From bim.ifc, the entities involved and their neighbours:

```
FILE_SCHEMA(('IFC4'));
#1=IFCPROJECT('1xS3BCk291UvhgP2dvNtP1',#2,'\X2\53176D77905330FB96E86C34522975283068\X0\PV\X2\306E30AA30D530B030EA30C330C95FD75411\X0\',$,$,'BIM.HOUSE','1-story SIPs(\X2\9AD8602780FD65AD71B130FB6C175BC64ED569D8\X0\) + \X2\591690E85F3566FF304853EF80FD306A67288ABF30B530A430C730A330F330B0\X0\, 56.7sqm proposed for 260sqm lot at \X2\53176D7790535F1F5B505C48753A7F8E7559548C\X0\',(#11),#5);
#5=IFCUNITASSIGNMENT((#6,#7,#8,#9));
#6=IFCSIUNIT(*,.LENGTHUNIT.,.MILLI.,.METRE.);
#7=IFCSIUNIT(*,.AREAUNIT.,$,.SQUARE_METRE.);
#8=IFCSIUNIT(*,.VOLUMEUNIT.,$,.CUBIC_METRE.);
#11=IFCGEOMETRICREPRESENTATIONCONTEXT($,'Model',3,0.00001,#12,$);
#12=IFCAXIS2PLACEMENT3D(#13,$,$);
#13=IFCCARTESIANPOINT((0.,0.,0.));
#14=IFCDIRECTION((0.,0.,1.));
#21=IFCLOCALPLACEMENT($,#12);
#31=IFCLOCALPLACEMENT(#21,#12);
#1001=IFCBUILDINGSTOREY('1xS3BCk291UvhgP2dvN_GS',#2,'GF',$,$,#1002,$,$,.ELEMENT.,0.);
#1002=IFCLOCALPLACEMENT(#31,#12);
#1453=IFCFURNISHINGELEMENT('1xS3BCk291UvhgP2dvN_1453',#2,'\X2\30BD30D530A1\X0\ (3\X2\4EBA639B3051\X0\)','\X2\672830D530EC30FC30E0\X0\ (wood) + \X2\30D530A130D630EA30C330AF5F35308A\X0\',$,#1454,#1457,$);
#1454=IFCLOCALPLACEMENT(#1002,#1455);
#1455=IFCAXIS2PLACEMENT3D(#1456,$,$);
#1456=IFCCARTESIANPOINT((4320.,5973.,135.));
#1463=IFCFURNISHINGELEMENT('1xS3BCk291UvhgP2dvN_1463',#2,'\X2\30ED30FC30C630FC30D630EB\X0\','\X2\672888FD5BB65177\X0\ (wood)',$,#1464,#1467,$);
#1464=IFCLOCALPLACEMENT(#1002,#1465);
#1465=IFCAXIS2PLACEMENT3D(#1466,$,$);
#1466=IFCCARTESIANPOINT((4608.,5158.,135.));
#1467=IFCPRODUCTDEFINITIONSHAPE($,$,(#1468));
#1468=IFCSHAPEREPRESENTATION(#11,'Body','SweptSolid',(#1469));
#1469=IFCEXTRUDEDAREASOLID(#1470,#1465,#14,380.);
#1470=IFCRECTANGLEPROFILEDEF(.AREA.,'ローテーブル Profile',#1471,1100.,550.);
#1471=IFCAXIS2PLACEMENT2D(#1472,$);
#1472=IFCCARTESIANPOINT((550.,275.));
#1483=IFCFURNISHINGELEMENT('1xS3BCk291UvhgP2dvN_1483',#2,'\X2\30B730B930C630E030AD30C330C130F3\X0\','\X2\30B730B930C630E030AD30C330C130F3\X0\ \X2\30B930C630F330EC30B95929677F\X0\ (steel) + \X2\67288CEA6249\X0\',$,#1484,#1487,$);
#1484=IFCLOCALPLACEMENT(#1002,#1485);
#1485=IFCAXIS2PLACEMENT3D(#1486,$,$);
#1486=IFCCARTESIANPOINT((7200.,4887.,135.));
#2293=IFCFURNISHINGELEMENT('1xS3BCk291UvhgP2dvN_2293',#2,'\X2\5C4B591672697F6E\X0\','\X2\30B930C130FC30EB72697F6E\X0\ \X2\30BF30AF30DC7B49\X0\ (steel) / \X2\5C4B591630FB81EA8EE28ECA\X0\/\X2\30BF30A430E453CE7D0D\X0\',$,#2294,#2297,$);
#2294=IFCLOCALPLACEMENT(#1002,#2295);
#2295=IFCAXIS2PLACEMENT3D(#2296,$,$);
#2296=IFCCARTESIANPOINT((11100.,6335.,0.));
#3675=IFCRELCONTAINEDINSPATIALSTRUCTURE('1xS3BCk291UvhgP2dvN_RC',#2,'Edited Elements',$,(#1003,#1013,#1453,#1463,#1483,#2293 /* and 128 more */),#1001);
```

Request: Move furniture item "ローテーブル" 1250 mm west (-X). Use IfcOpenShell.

```python
import ifcopenshell
import ifcopenshell.api.geometry
import ifcopenshell.util.placement
import ifcopenshell.util.unit

model = ifcopenshell.open("bim.ifc")
unit_scale = ifcopenshell.util.unit.calculate_unit_scale(model)

item = model.by_guid("1xS3BCk291UvhgP2dvN_1463")
matrix = ifcopenshell.util.placement.get_local_placement(item.ObjectPlacement)
matrix[0, 3] -= 1.25 / unit_scale
ifcopenshell.api.geometry.edit_object_placement(model, product=item, matrix=matrix, is_si=False)

print(ifcopenshell.util.placement.get_local_placement(item.ObjectPlacement).round(3) + 0.0)

model.write("bim_updated.ifc")
```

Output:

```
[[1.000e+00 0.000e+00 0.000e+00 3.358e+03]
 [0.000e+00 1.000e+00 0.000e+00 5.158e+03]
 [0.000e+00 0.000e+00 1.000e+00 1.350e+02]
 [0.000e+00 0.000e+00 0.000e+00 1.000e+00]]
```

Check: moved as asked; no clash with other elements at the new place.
